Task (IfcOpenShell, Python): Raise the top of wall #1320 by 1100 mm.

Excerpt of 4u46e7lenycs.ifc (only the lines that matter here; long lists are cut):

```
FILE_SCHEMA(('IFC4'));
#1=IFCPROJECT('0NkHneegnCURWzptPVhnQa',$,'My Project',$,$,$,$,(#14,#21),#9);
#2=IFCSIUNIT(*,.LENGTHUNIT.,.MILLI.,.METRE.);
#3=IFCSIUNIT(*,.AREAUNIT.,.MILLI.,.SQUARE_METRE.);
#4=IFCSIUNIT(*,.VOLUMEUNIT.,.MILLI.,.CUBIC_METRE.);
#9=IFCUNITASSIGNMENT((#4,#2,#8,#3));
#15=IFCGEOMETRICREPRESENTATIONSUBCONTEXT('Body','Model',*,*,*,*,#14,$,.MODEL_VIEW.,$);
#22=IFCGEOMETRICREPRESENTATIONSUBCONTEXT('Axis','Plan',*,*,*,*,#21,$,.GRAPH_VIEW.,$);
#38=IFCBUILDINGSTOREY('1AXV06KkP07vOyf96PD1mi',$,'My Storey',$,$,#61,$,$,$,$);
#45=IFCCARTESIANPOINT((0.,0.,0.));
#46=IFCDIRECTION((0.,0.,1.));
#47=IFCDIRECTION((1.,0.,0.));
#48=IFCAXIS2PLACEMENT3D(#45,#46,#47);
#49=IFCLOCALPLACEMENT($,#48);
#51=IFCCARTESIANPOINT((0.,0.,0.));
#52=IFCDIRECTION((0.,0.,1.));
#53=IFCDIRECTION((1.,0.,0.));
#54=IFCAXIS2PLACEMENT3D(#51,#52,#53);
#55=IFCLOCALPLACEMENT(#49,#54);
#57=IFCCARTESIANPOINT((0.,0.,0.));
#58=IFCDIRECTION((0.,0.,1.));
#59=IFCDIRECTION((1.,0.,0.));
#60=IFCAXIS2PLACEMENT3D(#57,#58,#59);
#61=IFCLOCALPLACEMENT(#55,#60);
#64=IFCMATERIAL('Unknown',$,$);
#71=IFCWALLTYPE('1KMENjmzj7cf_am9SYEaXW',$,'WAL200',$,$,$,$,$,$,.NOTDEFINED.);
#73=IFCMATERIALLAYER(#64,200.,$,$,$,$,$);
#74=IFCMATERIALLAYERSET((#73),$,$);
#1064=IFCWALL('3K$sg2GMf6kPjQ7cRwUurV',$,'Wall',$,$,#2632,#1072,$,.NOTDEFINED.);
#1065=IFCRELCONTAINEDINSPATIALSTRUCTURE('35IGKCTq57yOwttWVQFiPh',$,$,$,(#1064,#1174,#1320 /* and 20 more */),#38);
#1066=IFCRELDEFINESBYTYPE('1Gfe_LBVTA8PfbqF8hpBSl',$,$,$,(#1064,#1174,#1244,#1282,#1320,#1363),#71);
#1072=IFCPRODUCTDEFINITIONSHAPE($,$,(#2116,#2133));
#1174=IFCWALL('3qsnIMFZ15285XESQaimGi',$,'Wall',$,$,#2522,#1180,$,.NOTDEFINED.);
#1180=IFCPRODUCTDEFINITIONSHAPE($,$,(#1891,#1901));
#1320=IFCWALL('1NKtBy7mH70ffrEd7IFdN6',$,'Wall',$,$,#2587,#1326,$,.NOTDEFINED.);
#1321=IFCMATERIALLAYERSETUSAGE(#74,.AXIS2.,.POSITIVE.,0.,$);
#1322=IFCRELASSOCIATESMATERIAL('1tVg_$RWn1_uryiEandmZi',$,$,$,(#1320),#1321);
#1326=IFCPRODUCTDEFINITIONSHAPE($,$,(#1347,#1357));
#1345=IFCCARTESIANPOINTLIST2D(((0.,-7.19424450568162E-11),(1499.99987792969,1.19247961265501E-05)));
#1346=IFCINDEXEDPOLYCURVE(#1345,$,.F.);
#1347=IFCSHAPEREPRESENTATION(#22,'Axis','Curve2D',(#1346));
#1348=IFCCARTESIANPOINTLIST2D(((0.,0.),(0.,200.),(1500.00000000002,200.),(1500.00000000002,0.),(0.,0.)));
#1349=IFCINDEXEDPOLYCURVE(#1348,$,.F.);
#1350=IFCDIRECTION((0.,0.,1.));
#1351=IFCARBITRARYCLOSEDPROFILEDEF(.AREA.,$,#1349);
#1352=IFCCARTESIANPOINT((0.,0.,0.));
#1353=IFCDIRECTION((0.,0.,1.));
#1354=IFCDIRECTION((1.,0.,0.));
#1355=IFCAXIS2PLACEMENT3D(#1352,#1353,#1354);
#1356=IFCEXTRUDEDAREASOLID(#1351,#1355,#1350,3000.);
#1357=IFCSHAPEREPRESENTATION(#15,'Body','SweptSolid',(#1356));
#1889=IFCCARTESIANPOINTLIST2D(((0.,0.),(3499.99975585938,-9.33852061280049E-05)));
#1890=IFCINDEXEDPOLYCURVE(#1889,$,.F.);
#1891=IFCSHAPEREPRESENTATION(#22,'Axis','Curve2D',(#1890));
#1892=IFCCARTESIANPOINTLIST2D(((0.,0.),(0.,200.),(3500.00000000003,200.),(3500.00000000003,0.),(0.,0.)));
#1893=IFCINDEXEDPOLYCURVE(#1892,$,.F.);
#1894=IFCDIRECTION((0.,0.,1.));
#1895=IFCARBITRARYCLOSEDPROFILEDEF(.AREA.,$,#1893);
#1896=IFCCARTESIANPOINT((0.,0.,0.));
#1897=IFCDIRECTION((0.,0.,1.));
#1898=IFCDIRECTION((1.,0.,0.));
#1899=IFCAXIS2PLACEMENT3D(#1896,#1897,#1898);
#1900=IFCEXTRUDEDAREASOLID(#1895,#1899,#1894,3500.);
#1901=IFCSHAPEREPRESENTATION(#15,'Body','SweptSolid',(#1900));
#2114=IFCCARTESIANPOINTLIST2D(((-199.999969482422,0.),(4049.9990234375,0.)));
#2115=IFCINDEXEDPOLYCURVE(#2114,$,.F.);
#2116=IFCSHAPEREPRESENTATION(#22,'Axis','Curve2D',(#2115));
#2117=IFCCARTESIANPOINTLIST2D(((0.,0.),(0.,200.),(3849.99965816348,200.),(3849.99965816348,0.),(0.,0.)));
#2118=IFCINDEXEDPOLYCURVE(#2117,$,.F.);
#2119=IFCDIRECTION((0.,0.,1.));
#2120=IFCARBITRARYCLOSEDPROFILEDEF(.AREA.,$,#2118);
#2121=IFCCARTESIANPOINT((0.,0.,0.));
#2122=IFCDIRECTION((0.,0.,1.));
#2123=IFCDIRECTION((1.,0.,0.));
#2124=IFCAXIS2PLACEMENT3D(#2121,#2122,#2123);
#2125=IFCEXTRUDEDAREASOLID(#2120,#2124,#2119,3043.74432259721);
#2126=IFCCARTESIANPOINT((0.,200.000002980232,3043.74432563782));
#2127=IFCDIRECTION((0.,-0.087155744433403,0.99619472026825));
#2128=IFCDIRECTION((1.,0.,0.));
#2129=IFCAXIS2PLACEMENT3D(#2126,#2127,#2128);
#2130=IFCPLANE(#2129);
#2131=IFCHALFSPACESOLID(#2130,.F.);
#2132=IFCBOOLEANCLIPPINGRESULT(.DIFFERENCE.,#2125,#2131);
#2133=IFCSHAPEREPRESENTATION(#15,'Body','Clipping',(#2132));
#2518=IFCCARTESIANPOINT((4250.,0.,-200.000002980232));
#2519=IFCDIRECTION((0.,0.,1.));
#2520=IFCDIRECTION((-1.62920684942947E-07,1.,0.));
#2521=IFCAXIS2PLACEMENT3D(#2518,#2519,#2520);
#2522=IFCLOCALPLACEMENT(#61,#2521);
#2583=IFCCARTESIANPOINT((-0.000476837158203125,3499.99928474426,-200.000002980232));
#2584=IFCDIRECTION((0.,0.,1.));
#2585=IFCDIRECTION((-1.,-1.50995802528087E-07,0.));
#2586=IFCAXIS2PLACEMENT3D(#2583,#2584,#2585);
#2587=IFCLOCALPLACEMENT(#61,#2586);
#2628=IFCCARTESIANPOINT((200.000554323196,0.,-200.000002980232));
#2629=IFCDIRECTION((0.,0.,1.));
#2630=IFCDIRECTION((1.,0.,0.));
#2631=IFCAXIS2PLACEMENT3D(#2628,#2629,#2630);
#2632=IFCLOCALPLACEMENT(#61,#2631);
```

```python
import ifcopenshell
import ifcopenshell.geom
import ifcopenshell.util.representation
import ifcopenshell.util.shape

model = ifcopenshell.open("4u46e7lenycs.ifc")
settings = ifcopenshell.geom.settings()


def volume(element):
    """Net volume in cubic metres, openings subtracted."""
    shape = ifcopenshell.geom.create_shape(settings, element)
    return ifcopenshell.util.shape.get_volume(shape.geometry)


wall = model.by_guid("1NKtBy7mH70ffrEd7IFdN6")
before = volume(wall)

body = ifcopenshell.util.representation.get_representation(wall, "Model", "Body")
solid = body.Items[0]
old_height = solid.Depth
solid.Depth += 1100.0
after = volume(wall)

print(f"height {old_height:g} -> {solid.Depth:g}, volume {before:.3f} -> {after:.3f} m3")

model.write("4u46e7lenycs_rev.ifc")
```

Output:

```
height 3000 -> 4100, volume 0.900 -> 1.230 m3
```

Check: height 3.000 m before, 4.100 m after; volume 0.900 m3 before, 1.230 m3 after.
